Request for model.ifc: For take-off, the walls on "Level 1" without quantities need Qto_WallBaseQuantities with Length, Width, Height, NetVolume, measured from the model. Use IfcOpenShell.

First a look at what the model holds.

```python
import ifcopenshell
import ifcopenshell.util.element
import ifcopenshell.util.unit

model = ifcopenshell.open("model.ifc")
print(model.schema)
for unit_type in ("LENGTHUNIT", "AREAUNIT", "VOLUMEUNIT"):
    print(unit_type, ifcopenshell.util.unit.calculate_unit_scale(model, unit_type))
storey = next(s for s in model.by_type("IfcBuildingStorey") if s.Name == "Level 1")
walls = [e for e in ifcopenshell.util.element.get_decomposition(storey) if e.is_a("IfcWall")]
for e in sorted(walls, key=lambda e: e.id()):
    print(e.id(), e.is_a(), e.Name, list(ifcopenshell.util.element.get_psets(e, qtos_only=True)), sep=" | ")
```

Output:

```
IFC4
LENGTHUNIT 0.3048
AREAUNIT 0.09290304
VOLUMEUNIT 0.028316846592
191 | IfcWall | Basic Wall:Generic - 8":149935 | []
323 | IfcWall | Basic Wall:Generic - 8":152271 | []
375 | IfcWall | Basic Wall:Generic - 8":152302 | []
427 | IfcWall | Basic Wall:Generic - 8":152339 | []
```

```python
import ifcopenshell
import ifcopenshell.api.pset
import ifcopenshell.geom
import ifcopenshell.util.element
import ifcopenshell.util.shape
import ifcopenshell.util.unit

model = ifcopenshell.open("model.ifc")
unit_scale = ifcopenshell.util.unit.calculate_unit_scale(model)
volume_scale = ifcopenshell.util.unit.calculate_unit_scale(model, "VOLUMEUNIT")
settings = ifcopenshell.geom.settings()

storey = next(s for s in model.by_type("IfcBuildingStorey") if s.Name == "Level 1")
walls = [e for e in ifcopenshell.util.element.get_decomposition(storey) if e.is_a("IfcWall")]

for e in sorted(walls, key=lambda e: e.id()):
    if ifcopenshell.util.element.get_psets(e, qtos_only=True, should_inherit=False):
        continue
    # Geometry comes back in metres, in the element's own axes.
    shape = ifcopenshell.geom.create_shape(settings, e)
    values = {
        "Length": ifcopenshell.util.shape.get_x(shape.geometry) / unit_scale,
        "Width": ifcopenshell.util.shape.get_y(shape.geometry) / unit_scale,
        "Height": ifcopenshell.util.shape.get_z(shape.geometry) / unit_scale,
        "NetVolume": ifcopenshell.util.shape.get_volume(shape.geometry) / volume_scale,
    }
    qto = ifcopenshell.api.pset.add_qto(model, product=e, name="Qto_WallBaseQuantities")
    ifcopenshell.api.pset.edit_qto(model, qto=qto, properties=values)
    print(e.id(), {k: round(v, 3) for k, v in values.items()})

model.write("model_updated.ifc")
```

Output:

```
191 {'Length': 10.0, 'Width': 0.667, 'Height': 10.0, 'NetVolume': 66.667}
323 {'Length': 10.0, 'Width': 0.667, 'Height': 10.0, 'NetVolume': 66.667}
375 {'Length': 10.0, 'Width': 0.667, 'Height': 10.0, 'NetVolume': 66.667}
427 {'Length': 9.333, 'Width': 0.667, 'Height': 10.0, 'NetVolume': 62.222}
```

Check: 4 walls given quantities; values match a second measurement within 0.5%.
